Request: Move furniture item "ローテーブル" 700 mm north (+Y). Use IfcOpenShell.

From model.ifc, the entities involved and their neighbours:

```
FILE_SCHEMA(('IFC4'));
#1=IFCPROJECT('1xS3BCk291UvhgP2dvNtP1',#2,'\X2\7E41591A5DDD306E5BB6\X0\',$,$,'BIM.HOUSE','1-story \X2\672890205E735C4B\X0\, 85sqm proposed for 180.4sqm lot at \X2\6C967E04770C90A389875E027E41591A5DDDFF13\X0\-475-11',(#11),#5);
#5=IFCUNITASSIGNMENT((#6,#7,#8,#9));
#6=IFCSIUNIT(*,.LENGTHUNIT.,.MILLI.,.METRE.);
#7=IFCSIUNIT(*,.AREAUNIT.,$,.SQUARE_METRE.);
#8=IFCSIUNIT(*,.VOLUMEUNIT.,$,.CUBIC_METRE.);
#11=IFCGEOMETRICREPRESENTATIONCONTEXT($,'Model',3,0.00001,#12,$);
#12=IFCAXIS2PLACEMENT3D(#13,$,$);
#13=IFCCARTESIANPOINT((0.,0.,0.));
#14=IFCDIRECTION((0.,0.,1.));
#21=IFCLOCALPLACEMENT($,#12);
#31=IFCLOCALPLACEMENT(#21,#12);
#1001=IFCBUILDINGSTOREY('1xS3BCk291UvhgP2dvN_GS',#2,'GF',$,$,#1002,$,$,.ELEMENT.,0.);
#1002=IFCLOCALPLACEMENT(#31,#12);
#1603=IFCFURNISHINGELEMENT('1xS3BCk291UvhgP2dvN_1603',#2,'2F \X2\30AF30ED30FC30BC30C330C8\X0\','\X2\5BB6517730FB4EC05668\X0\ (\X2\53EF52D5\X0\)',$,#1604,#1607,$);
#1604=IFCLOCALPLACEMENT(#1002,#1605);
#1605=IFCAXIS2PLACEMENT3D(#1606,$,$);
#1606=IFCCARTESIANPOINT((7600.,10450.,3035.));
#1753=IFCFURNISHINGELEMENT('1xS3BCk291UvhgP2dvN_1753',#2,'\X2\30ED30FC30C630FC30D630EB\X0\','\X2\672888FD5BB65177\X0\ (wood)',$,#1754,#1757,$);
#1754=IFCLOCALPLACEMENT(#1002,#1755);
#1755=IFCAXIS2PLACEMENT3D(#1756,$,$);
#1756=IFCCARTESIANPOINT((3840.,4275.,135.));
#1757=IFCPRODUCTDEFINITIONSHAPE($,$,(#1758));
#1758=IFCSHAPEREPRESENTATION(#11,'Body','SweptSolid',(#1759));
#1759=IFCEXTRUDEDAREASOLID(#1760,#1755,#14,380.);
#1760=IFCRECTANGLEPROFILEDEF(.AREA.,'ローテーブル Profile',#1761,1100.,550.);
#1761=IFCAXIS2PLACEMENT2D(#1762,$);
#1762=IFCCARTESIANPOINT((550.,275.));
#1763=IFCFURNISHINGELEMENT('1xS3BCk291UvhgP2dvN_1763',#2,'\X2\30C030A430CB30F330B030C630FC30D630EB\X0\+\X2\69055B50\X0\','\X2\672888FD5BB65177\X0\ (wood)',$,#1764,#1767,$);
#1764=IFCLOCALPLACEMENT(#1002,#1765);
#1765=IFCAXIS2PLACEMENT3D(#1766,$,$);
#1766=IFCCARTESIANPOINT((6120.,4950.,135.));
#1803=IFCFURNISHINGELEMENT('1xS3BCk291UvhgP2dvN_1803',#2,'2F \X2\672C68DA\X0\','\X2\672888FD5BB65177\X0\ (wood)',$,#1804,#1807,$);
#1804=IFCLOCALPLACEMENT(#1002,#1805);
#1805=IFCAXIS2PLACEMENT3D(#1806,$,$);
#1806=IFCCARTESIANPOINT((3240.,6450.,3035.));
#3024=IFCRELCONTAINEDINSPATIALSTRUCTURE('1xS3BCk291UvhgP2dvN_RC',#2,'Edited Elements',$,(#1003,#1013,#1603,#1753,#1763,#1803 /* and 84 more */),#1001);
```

```python
import ifcopenshell
import ifcopenshell.api.geometry
import ifcopenshell.util.placement

model = ifcopenshell.open("model.ifc")

item = model.by_id(1753)
matrix = ifcopenshell.util.placement.get_local_placement(item.ObjectPlacement)
matrix[1, 3] += 700.0
ifcopenshell.api.geometry.edit_object_placement(model, product=item, matrix=matrix, is_si=False)

print(ifcopenshell.util.placement.get_local_placement(item.ObjectPlacement).round(3) + 0.0)

model.write("model_updated.ifc")
```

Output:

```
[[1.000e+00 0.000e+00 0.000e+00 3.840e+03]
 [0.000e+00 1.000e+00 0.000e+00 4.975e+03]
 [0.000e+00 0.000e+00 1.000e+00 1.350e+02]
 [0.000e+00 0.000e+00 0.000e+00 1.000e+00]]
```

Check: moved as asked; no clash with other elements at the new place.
